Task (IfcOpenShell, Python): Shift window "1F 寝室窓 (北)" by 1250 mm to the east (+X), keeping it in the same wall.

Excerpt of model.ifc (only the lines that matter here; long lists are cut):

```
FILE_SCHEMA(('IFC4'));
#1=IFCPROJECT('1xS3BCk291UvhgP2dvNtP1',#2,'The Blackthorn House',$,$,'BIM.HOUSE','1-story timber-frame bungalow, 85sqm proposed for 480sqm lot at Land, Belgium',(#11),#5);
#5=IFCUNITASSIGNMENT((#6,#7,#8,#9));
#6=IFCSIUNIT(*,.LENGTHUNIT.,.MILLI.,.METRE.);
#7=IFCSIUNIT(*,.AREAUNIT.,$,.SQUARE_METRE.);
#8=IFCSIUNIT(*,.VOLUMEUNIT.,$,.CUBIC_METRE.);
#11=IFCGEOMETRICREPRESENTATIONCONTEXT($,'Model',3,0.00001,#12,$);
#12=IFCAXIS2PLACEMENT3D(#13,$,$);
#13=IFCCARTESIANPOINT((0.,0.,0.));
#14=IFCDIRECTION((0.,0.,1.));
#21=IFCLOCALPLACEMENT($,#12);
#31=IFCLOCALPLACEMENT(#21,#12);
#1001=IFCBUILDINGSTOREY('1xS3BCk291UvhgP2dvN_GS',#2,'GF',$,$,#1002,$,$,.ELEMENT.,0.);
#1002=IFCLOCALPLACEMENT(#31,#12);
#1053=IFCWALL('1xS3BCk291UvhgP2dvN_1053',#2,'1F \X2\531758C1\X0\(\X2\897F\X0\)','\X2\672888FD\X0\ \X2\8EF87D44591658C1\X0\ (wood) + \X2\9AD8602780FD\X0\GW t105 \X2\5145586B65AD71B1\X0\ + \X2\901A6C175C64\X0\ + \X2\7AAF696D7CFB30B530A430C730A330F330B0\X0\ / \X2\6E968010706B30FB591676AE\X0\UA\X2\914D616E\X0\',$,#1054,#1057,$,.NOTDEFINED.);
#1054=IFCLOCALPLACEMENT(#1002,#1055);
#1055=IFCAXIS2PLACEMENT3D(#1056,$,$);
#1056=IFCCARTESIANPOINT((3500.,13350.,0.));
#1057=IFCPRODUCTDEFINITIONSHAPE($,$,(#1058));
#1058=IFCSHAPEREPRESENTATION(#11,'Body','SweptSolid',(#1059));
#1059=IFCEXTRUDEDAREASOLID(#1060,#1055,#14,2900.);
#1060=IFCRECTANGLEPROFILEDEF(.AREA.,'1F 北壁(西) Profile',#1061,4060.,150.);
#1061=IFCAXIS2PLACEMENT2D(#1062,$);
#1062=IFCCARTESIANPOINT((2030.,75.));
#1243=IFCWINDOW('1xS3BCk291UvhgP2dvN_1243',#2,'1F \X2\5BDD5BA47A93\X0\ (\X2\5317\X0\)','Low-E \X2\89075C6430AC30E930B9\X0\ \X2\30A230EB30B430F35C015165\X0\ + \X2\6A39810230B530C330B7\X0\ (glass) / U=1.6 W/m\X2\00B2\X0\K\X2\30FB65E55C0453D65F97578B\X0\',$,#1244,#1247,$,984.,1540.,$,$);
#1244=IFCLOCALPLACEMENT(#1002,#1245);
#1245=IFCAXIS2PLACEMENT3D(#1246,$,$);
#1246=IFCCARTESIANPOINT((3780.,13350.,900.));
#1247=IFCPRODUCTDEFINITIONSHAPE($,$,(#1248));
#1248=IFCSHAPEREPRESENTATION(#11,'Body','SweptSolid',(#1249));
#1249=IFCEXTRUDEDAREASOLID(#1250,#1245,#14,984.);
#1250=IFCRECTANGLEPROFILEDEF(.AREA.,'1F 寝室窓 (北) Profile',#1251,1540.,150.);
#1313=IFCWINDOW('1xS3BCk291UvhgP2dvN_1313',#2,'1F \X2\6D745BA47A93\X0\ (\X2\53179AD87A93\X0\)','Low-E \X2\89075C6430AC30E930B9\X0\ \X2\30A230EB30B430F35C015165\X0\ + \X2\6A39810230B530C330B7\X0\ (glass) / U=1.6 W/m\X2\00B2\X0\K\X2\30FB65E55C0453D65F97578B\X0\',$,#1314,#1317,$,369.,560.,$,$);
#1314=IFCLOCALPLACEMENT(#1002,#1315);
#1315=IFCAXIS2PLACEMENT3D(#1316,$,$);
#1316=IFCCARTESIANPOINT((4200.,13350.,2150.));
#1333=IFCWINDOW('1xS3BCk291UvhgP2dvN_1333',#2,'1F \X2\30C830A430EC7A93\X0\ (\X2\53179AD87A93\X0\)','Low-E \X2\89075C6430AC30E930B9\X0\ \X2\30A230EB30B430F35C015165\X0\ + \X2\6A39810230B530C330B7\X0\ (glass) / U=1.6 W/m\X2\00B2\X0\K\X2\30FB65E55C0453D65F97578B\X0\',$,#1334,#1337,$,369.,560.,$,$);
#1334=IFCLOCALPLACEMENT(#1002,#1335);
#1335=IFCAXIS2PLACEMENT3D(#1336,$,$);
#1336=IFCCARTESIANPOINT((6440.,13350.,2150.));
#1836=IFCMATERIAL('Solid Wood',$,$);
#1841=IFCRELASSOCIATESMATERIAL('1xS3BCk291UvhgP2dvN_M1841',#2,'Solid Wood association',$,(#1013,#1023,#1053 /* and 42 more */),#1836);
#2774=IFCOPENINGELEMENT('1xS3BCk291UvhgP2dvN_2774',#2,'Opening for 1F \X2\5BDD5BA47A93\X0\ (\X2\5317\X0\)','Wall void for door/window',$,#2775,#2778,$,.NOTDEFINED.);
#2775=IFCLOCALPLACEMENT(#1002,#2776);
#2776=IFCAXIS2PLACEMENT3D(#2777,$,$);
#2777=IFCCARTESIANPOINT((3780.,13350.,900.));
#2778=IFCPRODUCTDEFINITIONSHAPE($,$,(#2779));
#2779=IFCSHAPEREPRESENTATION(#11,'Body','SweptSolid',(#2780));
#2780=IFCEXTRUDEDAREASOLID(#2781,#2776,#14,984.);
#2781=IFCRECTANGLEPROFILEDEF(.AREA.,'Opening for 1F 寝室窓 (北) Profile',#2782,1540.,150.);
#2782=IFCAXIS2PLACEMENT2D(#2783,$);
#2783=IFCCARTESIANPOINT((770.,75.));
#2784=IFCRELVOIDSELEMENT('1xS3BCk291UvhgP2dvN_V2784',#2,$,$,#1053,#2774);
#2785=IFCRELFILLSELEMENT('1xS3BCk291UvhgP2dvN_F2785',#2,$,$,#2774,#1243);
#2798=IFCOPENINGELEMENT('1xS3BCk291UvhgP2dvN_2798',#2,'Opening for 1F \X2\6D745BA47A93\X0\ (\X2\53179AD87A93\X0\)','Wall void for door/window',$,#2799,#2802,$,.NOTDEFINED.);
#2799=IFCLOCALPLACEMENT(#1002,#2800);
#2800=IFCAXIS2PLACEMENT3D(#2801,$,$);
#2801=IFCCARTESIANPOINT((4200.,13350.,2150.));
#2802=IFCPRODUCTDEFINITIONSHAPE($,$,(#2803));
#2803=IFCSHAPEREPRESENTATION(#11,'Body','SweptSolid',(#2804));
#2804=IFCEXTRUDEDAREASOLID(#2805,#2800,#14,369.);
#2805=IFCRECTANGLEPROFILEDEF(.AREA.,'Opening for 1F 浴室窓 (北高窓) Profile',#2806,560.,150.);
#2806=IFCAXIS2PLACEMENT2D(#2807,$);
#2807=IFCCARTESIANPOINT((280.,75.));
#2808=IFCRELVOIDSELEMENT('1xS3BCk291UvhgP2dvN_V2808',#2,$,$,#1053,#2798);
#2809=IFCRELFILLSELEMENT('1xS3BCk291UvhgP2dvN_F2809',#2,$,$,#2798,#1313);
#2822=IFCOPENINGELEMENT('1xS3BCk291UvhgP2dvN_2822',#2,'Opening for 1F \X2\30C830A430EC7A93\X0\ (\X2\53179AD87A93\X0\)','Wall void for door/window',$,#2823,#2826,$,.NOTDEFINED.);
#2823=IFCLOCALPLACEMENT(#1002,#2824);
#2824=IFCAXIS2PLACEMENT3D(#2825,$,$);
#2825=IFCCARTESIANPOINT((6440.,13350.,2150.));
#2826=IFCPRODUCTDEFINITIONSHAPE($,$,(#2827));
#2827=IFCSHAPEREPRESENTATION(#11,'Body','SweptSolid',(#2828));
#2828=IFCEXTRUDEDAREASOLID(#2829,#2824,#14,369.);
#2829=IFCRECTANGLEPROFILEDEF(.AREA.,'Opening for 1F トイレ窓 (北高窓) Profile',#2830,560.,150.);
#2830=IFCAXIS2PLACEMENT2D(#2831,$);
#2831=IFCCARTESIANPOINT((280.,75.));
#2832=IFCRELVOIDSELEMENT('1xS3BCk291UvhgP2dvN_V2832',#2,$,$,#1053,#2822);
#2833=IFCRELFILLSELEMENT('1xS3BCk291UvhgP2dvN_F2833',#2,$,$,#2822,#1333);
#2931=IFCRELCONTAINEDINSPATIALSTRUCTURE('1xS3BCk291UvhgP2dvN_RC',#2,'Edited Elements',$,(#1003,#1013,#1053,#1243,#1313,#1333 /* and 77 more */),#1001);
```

```python
import ifcopenshell
import ifcopenshell.api.geometry
import ifcopenshell.util.placement

model = ifcopenshell.open("model.ifc")

window = model.by_guid("1xS3BCk291UvhgP2dvN_1243")
opening = window.FillsVoids[0].RelatingOpeningElement
wall = opening.VoidsElements[0].RelatingBuildingElement

wall_matrix = ifcopenshell.util.placement.get_local_placement(wall.ObjectPlacement)
shift = wall_matrix[:3, 0] * 1250.0
before = ifcopenshell.util.placement.get_local_placement(window.ObjectPlacement)[:3, 3].copy()

# The window is not placed relative to its opening, so move both.
for product in (opening, window):
    matrix = ifcopenshell.util.placement.get_local_placement(product.ObjectPlacement)
    matrix[:3, 3] += shift
    ifcopenshell.api.geometry.edit_object_placement(model, product=product, matrix=matrix, is_si=False)

after = ifcopenshell.util.placement.get_local_placement(window.ObjectPlacement)[:3, 3]
print("window moved by", (after - before).round(3) + 0.0)

model.write("model-out.ifc")
```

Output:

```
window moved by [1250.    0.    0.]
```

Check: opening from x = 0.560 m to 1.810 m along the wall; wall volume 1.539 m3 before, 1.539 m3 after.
